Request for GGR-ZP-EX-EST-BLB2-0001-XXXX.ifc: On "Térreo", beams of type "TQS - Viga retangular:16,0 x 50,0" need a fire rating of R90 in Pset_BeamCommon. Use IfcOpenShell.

First a look at what the model holds.

```python
import ifcopenshell
import ifcopenshell.util.element

model = ifcopenshell.open("GGR-ZP-EX-EST-BLB2-0001-XXXX.ifc")
print(model.schema)
storey = next(s for s in model.by_type("IfcBuildingStorey") if s.Name == "Térreo")
beams = [e for e in ifcopenshell.util.element.get_decomposition(storey) if e.is_a("IfcBeam")]
seen = {}
for e in beams:
    element_type = ifcopenshell.util.element.get_type(e)
    key = (element_type.Name if element_type != e and element_type else None, ifcopenshell.util.element.get_pset(e, "Pset_BeamCommon", "FireRating"))
    seen[key] = seen.get(key, 0) + 1
for (name, value), count in sorted(seen.items(), key=str):
    print(count, "x", name, "|", value)
```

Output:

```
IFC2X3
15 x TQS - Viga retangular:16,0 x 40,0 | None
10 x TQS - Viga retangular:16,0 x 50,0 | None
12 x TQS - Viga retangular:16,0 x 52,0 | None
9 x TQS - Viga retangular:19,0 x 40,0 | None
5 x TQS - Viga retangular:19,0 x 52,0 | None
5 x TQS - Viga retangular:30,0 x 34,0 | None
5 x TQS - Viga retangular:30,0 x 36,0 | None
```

```python
import ifcopenshell
import ifcopenshell.api.pset
import ifcopenshell.util.element

model = ifcopenshell.open("GGR-ZP-EX-EST-BLB2-0001-XXXX.ifc")

storey = next(s for s in model.by_type("IfcBuildingStorey") if s.Name == "Térreo")
beams = [e for e in ifcopenshell.util.element.get_decomposition(storey) if e.is_a("IfcBeam")]

count = 0
for e in beams:
    element_type = ifcopenshell.util.element.get_type(e)
    if element_type in (None, e) or element_type.Name != "TQS - Viga retangular:16,0 x 50,0":
        continue
    # add_pset returns the element's existing set when there is one.
    pset = ifcopenshell.api.pset.add_pset(model, product=e, name="Pset_BeamCommon")
    ifcopenshell.api.pset.edit_pset(model, pset=pset, properties={"FireRating": "R90"})
    count += 1

print(count, "beams updated")

model.write("GGR-ZP-EX-EST-BLB2-0001-XXXX_edited.ifc")
```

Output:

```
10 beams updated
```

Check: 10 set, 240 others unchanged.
